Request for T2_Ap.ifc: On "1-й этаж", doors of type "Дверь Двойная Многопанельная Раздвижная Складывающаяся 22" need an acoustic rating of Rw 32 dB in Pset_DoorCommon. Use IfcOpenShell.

First a look at what the model holds.

```python
import ifcopenshell
import ifcopenshell.util.element

model = ifcopenshell.open("T2_Ap.ifc")
print(model.schema)
storey = next(s for s in model.by_type("IfcBuildingStorey") if s.Name == "1-й этаж")
doors = [e for e in ifcopenshell.util.element.get_decomposition(storey) if e.is_a("IfcDoor")]
seen = {}
for e in doors:
    element_type = ifcopenshell.util.element.get_type(e)
    key = (element_type.Name if element_type != e and element_type else None, ifcopenshell.util.element.get_pset(e, "Pset_DoorCommon", "AcousticRating"))
    seen[key] = seen.get(key, 0) + 1
for (name, value), count in sorted(seen.items(), key=str):
    print(count, "x", name, "|", value)
```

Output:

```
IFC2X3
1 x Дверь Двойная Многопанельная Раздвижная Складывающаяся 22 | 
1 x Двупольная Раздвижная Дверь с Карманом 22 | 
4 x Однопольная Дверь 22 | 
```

```python
import ifcopenshell
import ifcopenshell.api.pset
import ifcopenshell.util.element

model = ifcopenshell.open("T2_Ap.ifc")

storey = next(s for s in model.by_type("IfcBuildingStorey") if s.Name == "1-й этаж")
doors = [e for e in ifcopenshell.util.element.get_decomposition(storey) if e.is_a("IfcDoor")]

count = 0
for e in doors:
    element_type = ifcopenshell.util.element.get_type(e)
    if element_type in (None, e) or element_type.Name != "Дверь Двойная Многопанельная Раздвижная Складывающаяся 22":
        continue
    # add_pset returns the element's existing set when there is one.
    pset = ifcopenshell.api.pset.add_pset(model, product=e, name="Pset_DoorCommon")
    ifcopenshell.api.pset.edit_pset(model, pset=pset, properties={"AcousticRating": "Rw 32 dB"})
    count += 1

print(count, "doors updated")

model.write("T2_Ap_v2.ifc")
```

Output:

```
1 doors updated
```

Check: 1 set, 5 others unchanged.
